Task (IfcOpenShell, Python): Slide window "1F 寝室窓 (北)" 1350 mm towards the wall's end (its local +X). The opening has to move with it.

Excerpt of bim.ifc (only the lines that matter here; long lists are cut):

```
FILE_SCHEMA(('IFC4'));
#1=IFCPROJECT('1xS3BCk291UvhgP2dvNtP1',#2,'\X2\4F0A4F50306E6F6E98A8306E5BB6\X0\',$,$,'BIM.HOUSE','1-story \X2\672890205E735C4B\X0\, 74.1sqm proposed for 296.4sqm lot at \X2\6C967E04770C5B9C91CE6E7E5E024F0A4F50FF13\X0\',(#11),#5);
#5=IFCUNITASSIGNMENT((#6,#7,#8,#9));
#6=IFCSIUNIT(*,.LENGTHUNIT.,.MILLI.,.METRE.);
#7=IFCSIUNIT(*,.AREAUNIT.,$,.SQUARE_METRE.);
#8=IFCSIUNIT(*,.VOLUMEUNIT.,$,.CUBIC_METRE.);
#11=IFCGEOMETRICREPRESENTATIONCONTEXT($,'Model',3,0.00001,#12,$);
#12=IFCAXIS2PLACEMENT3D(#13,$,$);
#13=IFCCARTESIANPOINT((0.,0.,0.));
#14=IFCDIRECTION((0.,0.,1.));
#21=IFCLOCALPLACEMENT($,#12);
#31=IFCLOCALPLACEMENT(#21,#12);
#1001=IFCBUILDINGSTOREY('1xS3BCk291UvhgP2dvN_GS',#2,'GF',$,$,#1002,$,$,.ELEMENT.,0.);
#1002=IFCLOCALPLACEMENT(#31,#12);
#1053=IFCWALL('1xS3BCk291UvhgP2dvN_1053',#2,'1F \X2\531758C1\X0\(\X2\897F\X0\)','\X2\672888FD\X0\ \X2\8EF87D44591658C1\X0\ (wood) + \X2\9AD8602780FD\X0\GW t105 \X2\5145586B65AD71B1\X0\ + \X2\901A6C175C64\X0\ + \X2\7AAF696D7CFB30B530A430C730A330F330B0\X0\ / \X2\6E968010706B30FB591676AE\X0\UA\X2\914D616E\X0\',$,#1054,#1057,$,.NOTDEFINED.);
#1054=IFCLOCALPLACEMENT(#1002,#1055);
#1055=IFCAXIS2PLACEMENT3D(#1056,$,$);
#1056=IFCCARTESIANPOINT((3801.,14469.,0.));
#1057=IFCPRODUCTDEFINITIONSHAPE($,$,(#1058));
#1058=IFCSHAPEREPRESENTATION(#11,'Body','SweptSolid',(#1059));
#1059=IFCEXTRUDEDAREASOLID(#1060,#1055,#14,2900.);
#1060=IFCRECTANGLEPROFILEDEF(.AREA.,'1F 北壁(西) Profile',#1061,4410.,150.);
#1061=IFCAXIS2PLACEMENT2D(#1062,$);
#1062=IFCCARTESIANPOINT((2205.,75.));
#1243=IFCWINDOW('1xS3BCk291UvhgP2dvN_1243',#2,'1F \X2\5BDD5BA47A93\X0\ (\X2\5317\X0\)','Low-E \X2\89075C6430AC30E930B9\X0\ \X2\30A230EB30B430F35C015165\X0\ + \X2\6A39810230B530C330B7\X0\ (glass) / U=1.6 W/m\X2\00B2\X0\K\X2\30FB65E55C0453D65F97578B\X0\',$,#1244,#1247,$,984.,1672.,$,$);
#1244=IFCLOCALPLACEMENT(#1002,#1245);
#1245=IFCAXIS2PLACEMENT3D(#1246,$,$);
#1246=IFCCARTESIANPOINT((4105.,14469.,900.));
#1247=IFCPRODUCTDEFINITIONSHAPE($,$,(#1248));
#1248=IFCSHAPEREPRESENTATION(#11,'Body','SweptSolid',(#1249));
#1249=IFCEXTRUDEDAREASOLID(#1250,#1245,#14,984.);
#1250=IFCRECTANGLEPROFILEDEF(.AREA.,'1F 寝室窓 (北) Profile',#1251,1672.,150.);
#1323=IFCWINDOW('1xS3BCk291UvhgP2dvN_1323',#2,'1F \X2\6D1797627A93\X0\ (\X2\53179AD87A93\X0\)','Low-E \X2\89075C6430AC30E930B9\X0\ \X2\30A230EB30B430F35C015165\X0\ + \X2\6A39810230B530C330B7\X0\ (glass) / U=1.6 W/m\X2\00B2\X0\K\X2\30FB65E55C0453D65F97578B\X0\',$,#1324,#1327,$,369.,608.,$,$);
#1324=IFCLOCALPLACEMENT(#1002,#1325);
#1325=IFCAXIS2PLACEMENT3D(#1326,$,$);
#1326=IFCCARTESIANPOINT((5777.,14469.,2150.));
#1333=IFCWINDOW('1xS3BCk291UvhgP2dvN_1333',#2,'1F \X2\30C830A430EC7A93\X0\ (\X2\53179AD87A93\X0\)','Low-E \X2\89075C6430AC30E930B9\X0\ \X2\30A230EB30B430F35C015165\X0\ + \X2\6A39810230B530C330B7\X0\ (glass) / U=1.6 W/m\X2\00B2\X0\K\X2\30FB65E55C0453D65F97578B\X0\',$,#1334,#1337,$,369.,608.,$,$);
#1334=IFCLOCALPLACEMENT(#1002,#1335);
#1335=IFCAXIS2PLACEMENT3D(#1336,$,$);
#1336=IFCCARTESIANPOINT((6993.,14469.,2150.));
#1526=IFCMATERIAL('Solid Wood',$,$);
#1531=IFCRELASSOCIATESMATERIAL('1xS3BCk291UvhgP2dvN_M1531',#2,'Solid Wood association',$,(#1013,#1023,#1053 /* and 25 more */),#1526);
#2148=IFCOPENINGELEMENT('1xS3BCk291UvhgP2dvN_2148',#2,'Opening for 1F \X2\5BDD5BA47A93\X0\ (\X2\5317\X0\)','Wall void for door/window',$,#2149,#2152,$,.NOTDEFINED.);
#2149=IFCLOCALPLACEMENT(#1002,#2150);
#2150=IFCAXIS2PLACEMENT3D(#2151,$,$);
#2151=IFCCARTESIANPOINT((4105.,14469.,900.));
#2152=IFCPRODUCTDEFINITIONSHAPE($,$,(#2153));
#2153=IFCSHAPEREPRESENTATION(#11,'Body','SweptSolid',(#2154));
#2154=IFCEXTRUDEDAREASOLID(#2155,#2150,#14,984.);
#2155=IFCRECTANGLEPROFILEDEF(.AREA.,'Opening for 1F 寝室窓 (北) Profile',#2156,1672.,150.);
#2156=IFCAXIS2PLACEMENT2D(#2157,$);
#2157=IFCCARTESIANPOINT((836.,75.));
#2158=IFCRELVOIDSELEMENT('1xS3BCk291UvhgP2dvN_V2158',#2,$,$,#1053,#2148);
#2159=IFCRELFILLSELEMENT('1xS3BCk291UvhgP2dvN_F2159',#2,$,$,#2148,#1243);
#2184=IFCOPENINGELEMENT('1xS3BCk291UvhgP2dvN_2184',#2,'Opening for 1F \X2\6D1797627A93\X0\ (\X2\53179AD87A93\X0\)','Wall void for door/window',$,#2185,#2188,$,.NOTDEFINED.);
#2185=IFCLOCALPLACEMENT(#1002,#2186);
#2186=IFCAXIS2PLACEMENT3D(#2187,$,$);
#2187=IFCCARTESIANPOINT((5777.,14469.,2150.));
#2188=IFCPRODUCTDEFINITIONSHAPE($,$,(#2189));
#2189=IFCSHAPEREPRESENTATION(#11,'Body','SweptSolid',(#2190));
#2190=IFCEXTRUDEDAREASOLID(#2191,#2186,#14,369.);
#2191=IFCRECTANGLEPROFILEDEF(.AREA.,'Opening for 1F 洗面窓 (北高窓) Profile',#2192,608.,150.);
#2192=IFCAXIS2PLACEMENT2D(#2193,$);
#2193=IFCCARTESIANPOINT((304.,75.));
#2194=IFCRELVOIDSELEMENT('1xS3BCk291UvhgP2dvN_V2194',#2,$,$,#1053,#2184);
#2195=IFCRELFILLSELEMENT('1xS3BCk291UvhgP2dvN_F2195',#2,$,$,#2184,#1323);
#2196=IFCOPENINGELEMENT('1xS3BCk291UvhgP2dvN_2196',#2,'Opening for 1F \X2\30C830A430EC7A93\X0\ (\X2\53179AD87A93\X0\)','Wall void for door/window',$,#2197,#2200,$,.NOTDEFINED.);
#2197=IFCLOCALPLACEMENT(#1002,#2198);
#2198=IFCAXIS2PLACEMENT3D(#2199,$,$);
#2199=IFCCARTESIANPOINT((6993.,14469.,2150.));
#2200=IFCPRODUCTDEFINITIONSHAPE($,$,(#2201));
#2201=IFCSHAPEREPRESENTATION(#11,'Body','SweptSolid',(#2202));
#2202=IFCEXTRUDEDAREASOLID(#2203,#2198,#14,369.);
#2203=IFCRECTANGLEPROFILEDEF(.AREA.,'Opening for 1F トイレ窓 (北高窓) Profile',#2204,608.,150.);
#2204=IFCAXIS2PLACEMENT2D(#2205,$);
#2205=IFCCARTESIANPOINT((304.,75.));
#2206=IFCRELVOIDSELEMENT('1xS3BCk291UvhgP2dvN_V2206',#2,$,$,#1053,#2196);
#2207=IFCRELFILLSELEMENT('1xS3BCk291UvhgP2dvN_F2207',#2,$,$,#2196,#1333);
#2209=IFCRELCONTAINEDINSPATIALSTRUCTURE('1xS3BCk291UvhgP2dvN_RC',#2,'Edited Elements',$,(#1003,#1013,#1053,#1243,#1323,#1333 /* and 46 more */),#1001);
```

```python
import ifcopenshell
import ifcopenshell.api.geometry
import ifcopenshell.util.placement

model = ifcopenshell.open("bim.ifc")

window = model.by_guid("1xS3BCk291UvhgP2dvN_1243")
opening = window.FillsVoids[0].RelatingOpeningElement
wall = opening.VoidsElements[0].RelatingBuildingElement

wall_matrix = ifcopenshell.util.placement.get_local_placement(wall.ObjectPlacement)
shift = wall_matrix[:3, 0] * 1350.0
before = ifcopenshell.util.placement.get_local_placement(window.ObjectPlacement)[:3, 3].copy()

# The window is not placed relative to its opening, so move both.
for product in (opening, window):
    matrix = ifcopenshell.util.placement.get_local_placement(product.ObjectPlacement)
    matrix[:3, 3] += shift
    ifcopenshell.api.geometry.edit_object_placement(model, product=product, matrix=matrix, is_si=False)

after = ifcopenshell.util.placement.get_local_placement(window.ObjectPlacement)[:3, 3]
print("window moved by", (after - before).round(3) + 0.0)

model.write("bim_v2.ifc")
```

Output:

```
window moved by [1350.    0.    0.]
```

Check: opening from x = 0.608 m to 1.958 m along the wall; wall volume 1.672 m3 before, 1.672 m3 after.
